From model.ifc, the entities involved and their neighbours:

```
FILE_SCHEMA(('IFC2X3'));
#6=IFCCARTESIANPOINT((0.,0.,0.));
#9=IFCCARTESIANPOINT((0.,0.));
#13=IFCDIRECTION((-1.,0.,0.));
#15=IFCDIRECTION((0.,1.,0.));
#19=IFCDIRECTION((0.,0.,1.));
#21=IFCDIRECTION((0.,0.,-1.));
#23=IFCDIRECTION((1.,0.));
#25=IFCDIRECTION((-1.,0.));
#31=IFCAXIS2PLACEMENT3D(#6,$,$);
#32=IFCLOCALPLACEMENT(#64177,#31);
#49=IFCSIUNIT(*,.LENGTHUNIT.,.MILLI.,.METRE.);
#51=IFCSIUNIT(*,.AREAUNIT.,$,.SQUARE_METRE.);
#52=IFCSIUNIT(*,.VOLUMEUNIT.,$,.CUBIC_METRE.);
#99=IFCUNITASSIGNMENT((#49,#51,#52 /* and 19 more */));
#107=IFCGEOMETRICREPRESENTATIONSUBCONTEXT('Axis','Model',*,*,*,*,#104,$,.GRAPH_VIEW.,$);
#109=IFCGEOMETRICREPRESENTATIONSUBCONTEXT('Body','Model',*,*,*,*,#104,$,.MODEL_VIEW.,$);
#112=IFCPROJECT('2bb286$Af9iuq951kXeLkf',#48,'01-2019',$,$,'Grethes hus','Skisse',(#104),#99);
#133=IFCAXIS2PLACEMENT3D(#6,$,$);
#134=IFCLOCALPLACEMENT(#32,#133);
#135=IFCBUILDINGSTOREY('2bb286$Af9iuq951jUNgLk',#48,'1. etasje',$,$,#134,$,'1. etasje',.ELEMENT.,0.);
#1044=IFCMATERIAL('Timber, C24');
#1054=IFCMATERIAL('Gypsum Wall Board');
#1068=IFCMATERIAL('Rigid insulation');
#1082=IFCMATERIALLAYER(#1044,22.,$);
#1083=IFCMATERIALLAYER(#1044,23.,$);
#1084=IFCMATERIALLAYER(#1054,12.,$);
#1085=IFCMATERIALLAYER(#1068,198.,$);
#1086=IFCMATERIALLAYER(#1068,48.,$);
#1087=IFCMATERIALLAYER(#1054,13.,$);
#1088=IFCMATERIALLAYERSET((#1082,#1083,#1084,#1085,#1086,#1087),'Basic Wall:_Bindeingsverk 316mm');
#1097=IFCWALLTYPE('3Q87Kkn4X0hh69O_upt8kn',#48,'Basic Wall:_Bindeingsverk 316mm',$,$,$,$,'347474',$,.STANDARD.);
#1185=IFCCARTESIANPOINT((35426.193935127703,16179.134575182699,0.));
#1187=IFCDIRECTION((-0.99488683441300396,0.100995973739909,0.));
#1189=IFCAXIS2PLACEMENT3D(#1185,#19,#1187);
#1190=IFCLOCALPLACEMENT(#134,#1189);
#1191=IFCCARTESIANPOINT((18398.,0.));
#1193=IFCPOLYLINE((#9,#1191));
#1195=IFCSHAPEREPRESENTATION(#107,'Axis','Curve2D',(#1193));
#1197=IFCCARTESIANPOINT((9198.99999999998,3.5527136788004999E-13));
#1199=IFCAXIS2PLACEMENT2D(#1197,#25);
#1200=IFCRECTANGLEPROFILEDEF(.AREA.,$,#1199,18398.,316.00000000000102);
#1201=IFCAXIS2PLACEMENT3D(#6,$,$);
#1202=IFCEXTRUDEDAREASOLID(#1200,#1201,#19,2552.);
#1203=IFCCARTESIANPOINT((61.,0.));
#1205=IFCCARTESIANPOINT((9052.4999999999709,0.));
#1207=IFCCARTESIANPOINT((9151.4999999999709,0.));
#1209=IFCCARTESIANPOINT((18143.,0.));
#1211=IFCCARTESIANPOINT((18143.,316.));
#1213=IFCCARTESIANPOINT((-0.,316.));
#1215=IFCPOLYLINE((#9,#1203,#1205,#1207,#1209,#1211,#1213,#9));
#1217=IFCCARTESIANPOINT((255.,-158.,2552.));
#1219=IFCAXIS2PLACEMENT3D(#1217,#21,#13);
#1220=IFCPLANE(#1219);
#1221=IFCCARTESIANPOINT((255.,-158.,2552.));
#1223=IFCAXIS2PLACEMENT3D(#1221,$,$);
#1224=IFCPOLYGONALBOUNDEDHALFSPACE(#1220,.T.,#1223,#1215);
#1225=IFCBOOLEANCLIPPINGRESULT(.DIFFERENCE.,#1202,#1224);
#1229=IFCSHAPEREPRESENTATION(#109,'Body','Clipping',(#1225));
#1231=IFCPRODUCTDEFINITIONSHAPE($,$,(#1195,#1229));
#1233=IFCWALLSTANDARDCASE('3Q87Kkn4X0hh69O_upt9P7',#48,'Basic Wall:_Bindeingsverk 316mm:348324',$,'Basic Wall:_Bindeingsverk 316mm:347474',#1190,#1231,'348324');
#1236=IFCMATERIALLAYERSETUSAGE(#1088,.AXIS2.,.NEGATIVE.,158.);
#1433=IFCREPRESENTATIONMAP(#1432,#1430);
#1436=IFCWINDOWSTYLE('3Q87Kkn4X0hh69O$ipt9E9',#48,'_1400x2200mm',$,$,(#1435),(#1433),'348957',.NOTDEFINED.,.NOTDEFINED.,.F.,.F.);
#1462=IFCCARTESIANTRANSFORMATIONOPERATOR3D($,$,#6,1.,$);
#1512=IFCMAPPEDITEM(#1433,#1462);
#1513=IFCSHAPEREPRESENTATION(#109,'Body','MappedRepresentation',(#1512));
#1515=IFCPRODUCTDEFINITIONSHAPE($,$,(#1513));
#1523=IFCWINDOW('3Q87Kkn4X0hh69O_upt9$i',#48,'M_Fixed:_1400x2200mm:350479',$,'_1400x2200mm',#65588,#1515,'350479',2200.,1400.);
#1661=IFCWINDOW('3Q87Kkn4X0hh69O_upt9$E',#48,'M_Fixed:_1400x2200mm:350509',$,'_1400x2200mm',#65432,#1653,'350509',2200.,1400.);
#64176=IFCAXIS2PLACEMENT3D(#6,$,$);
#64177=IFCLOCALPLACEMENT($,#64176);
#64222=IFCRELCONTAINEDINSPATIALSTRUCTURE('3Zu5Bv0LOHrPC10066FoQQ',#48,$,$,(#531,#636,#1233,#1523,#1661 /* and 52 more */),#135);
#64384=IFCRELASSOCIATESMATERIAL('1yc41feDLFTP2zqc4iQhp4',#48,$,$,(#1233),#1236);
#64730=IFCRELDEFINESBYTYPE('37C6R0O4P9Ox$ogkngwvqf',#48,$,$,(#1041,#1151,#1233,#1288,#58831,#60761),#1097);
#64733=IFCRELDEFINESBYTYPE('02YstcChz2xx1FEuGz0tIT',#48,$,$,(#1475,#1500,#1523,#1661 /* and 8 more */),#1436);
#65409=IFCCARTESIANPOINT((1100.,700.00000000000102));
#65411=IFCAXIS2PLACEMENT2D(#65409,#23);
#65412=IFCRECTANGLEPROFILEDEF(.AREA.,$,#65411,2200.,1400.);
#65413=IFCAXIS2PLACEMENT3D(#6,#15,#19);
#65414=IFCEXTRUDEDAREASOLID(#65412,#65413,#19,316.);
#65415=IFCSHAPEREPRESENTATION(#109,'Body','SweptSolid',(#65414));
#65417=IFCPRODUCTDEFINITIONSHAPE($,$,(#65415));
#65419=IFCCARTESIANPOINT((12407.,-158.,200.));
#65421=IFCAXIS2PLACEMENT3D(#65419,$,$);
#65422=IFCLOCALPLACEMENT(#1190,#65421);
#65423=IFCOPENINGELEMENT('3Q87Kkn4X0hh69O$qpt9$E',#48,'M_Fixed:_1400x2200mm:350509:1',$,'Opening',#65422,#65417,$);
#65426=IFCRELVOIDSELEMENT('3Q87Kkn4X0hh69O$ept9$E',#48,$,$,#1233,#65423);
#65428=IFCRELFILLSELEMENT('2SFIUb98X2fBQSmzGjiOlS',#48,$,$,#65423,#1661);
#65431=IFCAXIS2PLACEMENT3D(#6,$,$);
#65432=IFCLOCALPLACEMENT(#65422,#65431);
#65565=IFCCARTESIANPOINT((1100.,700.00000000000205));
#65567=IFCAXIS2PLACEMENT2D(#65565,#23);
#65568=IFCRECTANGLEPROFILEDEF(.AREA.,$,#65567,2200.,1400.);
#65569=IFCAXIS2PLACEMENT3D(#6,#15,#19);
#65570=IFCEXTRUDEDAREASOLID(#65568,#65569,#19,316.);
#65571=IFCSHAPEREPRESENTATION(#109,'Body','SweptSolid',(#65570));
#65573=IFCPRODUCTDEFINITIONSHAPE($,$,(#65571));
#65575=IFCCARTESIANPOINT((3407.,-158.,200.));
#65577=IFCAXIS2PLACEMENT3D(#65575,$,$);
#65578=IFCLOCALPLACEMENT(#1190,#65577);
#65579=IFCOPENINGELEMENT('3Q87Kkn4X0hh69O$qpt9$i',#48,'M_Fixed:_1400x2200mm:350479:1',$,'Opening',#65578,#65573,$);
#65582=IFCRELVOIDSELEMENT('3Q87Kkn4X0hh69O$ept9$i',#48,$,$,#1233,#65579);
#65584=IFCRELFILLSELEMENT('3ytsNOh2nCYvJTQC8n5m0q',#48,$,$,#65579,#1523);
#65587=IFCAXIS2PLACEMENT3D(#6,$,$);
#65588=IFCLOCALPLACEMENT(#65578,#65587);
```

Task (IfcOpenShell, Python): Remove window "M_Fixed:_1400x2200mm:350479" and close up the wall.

```python
import ifcopenshell
import ifcopenshell.api.feature
import ifcopenshell.api.root
import ifcopenshell.geom
import ifcopenshell.util.shape

model = ifcopenshell.open("model.ifc")
settings = ifcopenshell.geom.settings()


def volume(element):
    """Net volume in cubic metres, openings subtracted."""
    shape = ifcopenshell.geom.create_shape(settings, element)
    return ifcopenshell.util.shape.get_volume(shape.geometry)


window = model.by_id(1523)
opening = window.FillsVoids[0].RelatingOpeningElement
wall = opening.VoidsElements[0].RelatingBuildingElement
before = volume(wall)

ifcopenshell.api.root.remove_product(model, product=window)
ifcopenshell.api.feature.remove_feature(model, feature=opening)

after = volume(wall)

print(f"wall volume {before:.3f} -> {after:.3f} m3")

model.write("model_edited.ifc")
```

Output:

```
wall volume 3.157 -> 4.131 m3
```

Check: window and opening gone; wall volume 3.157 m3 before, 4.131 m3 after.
